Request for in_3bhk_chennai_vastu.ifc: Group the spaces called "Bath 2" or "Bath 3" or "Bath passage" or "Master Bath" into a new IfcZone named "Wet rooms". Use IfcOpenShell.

First a look at what the model holds.

```python
import ifcopenshell

model = ifcopenshell.open("in_3bhk_chennai_vastu.ifc")
print(model.schema)
seen = {}
for space in model.by_type("IfcSpace"):
    seen[space.LongName] = seen.get(space.LongName, 0) + 1
for name, count in sorted(seen.items(), key=str):
    print(count, "x", name)
print("zones:", [z.Name for z in model.by_type("IfcZone")][:20])
```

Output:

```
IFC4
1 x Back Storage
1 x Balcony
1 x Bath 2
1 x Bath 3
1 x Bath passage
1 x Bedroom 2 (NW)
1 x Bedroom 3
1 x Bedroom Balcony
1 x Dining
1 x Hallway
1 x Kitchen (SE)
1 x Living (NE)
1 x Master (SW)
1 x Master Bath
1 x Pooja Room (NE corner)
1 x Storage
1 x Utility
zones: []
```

```python
import ifcopenshell
import ifcopenshell.api.group
import ifcopenshell.api.root

model = ifcopenshell.open("in_3bhk_chennai_vastu.ifc")

names = {"Bath 2", "Bath 3", "Bath passage", "Master Bath"}
spaces = [s for s in model.by_type("IfcSpace") if s.LongName in names]

zone = ifcopenshell.api.root.create_entity(model, ifc_class="IfcZone", name="Wet rooms")
ifcopenshell.api.group.assign_group(model, products=spaces, group=zone)
print(len(spaces), "spaces in", zone.Name)

model.write("in_3bhk_chennai_vastu_updated.ifc")
```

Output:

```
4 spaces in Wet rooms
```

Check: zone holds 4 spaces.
